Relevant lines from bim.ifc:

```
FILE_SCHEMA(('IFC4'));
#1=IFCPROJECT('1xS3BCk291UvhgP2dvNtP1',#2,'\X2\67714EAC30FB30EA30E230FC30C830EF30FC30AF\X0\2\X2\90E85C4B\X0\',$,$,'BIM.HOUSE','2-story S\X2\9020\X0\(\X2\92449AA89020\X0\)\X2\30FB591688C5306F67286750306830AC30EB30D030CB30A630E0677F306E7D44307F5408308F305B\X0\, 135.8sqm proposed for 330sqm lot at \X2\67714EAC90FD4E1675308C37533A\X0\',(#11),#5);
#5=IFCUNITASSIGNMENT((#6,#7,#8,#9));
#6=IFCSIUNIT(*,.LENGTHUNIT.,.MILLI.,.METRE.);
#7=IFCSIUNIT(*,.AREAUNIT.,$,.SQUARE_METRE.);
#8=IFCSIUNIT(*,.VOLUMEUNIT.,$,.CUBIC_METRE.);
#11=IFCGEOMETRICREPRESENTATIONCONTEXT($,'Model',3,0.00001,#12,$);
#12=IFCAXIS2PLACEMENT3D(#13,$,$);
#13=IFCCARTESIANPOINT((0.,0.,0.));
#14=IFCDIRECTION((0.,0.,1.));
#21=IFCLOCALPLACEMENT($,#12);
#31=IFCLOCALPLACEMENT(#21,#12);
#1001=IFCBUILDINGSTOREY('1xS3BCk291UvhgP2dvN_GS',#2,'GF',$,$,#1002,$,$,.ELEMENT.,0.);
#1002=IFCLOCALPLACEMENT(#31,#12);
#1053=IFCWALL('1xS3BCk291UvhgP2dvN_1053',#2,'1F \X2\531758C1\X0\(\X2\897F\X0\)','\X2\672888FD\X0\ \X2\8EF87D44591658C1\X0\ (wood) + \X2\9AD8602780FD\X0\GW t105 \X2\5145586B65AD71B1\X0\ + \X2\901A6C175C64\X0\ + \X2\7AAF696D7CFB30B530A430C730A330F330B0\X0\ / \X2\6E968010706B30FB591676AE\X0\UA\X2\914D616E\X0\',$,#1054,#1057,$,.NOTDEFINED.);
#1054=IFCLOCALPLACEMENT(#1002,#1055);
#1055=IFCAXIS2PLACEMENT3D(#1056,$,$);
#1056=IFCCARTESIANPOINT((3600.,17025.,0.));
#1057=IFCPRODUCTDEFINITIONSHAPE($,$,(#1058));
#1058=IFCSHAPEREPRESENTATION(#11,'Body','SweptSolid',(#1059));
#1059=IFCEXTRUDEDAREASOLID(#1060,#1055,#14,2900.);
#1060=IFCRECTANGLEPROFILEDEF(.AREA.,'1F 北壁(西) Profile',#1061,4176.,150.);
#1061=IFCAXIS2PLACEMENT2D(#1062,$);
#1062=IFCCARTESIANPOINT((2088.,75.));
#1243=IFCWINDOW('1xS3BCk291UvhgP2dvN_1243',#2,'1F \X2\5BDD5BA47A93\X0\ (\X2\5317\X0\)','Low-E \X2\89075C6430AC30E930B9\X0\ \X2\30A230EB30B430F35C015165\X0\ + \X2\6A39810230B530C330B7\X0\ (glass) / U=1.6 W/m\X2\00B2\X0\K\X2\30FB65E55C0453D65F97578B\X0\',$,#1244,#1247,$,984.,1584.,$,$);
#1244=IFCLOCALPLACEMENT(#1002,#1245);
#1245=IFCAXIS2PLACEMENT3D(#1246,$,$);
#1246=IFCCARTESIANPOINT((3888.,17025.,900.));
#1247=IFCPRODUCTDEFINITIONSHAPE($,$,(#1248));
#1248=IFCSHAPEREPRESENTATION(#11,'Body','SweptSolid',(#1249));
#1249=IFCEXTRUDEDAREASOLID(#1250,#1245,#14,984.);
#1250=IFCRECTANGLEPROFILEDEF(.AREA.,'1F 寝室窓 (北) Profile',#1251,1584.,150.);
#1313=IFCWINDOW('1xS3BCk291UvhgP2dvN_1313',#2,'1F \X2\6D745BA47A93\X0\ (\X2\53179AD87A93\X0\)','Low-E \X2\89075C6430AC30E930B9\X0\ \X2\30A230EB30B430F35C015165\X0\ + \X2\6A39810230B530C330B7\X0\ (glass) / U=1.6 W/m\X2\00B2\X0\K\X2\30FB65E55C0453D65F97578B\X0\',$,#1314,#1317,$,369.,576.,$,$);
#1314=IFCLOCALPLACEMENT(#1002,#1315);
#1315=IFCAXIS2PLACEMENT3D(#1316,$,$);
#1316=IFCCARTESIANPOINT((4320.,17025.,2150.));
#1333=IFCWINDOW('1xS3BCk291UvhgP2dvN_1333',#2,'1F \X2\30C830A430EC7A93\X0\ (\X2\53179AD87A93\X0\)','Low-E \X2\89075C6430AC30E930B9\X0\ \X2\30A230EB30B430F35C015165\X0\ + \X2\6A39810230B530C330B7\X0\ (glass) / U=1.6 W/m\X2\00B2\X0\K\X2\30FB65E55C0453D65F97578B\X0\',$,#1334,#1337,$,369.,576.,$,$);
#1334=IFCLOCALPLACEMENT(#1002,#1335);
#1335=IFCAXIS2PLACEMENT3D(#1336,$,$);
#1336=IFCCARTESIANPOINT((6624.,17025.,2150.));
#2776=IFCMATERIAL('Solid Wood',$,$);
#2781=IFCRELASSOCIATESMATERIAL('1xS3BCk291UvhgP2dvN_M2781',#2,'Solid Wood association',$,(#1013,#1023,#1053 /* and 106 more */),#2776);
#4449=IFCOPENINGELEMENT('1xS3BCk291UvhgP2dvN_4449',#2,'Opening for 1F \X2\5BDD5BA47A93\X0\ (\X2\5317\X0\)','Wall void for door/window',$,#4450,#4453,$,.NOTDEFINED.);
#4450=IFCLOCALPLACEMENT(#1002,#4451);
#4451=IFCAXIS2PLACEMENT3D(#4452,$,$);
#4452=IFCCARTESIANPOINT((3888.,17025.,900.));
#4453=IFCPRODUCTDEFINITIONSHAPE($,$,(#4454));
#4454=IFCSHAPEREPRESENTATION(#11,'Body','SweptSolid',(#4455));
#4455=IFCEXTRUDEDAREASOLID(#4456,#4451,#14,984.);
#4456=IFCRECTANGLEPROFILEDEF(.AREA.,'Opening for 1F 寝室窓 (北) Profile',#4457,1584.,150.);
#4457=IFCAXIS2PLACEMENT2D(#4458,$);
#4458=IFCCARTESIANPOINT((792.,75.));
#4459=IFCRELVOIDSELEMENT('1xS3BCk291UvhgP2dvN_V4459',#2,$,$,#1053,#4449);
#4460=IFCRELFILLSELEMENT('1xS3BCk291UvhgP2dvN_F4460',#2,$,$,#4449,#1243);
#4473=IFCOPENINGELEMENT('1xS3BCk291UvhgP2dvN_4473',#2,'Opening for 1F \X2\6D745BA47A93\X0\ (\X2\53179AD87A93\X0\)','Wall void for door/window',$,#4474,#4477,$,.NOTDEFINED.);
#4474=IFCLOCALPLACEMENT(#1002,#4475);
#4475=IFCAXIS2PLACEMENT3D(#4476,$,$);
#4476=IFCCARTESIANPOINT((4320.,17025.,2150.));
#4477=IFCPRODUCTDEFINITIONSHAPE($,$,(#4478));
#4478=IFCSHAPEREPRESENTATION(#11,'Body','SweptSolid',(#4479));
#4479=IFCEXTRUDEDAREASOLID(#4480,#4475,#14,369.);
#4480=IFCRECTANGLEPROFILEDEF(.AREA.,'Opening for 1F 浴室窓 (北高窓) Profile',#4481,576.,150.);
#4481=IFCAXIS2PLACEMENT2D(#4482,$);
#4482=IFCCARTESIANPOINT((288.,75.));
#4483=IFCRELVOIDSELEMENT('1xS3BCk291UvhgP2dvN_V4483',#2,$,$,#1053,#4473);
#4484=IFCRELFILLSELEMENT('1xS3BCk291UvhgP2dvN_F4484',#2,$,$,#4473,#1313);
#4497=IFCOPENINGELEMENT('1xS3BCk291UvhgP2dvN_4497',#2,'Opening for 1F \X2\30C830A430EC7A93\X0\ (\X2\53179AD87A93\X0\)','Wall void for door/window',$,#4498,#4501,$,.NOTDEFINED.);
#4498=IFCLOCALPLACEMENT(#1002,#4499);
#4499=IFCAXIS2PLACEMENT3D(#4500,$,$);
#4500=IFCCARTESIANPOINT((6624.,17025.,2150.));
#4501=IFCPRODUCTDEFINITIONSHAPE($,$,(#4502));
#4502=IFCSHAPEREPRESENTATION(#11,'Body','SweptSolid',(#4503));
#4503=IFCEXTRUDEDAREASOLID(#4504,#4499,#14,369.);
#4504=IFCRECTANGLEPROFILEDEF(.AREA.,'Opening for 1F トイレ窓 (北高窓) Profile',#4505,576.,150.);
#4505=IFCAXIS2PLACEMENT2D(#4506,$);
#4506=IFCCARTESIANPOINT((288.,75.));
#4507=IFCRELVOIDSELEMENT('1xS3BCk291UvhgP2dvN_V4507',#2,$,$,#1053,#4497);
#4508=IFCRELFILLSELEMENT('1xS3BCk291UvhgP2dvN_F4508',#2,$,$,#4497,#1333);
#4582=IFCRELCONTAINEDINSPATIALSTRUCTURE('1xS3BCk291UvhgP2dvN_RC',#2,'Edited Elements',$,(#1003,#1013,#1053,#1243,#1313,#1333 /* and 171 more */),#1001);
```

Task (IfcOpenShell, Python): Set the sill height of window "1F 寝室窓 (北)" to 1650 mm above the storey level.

```python
import numpy as np
import ifcopenshell
import ifcopenshell.api.geometry
import ifcopenshell.geom
import ifcopenshell.util.element
import ifcopenshell.util.placement
import ifcopenshell.util.shape
import ifcopenshell.util.unit

model = ifcopenshell.open("bim.ifc")
unit_scale = ifcopenshell.util.unit.calculate_unit_scale(model)

window = model.by_id(1243)
opening = window.FillsVoids[0].RelatingOpeningElement
storey = ifcopenshell.util.element.get_container(window, ifc_class="IfcBuildingStorey")
level = ifcopenshell.util.placement.get_local_placement(storey.ObjectPlacement)[2, 3]

# The opening's origin need not be at the sill, so measure its lowest point.
shape = ifcopenshell.geom.create_shape(ifcopenshell.geom.settings(), opening)
bottom = ifcopenshell.util.shape.get_shape_bottom_elevation(shape, shape.geometry) / unit_scale
dz = level + 1.65 / unit_scale - bottom

shift = np.array([0.0, 0.0, dz])
# The window is not placed relative to its opening, so move both.
for product in (opening, window):
    matrix = ifcopenshell.util.placement.get_local_placement(product.ObjectPlacement)
    matrix[:3, 3] += shift
    ifcopenshell.api.geometry.edit_object_placement(model, product=product, matrix=matrix, is_si=False)

print(f"moved by {dz * unit_scale:+.3f} m")

model.write("bim_updated.ifc")
```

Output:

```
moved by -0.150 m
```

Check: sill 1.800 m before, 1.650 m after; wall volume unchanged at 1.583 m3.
